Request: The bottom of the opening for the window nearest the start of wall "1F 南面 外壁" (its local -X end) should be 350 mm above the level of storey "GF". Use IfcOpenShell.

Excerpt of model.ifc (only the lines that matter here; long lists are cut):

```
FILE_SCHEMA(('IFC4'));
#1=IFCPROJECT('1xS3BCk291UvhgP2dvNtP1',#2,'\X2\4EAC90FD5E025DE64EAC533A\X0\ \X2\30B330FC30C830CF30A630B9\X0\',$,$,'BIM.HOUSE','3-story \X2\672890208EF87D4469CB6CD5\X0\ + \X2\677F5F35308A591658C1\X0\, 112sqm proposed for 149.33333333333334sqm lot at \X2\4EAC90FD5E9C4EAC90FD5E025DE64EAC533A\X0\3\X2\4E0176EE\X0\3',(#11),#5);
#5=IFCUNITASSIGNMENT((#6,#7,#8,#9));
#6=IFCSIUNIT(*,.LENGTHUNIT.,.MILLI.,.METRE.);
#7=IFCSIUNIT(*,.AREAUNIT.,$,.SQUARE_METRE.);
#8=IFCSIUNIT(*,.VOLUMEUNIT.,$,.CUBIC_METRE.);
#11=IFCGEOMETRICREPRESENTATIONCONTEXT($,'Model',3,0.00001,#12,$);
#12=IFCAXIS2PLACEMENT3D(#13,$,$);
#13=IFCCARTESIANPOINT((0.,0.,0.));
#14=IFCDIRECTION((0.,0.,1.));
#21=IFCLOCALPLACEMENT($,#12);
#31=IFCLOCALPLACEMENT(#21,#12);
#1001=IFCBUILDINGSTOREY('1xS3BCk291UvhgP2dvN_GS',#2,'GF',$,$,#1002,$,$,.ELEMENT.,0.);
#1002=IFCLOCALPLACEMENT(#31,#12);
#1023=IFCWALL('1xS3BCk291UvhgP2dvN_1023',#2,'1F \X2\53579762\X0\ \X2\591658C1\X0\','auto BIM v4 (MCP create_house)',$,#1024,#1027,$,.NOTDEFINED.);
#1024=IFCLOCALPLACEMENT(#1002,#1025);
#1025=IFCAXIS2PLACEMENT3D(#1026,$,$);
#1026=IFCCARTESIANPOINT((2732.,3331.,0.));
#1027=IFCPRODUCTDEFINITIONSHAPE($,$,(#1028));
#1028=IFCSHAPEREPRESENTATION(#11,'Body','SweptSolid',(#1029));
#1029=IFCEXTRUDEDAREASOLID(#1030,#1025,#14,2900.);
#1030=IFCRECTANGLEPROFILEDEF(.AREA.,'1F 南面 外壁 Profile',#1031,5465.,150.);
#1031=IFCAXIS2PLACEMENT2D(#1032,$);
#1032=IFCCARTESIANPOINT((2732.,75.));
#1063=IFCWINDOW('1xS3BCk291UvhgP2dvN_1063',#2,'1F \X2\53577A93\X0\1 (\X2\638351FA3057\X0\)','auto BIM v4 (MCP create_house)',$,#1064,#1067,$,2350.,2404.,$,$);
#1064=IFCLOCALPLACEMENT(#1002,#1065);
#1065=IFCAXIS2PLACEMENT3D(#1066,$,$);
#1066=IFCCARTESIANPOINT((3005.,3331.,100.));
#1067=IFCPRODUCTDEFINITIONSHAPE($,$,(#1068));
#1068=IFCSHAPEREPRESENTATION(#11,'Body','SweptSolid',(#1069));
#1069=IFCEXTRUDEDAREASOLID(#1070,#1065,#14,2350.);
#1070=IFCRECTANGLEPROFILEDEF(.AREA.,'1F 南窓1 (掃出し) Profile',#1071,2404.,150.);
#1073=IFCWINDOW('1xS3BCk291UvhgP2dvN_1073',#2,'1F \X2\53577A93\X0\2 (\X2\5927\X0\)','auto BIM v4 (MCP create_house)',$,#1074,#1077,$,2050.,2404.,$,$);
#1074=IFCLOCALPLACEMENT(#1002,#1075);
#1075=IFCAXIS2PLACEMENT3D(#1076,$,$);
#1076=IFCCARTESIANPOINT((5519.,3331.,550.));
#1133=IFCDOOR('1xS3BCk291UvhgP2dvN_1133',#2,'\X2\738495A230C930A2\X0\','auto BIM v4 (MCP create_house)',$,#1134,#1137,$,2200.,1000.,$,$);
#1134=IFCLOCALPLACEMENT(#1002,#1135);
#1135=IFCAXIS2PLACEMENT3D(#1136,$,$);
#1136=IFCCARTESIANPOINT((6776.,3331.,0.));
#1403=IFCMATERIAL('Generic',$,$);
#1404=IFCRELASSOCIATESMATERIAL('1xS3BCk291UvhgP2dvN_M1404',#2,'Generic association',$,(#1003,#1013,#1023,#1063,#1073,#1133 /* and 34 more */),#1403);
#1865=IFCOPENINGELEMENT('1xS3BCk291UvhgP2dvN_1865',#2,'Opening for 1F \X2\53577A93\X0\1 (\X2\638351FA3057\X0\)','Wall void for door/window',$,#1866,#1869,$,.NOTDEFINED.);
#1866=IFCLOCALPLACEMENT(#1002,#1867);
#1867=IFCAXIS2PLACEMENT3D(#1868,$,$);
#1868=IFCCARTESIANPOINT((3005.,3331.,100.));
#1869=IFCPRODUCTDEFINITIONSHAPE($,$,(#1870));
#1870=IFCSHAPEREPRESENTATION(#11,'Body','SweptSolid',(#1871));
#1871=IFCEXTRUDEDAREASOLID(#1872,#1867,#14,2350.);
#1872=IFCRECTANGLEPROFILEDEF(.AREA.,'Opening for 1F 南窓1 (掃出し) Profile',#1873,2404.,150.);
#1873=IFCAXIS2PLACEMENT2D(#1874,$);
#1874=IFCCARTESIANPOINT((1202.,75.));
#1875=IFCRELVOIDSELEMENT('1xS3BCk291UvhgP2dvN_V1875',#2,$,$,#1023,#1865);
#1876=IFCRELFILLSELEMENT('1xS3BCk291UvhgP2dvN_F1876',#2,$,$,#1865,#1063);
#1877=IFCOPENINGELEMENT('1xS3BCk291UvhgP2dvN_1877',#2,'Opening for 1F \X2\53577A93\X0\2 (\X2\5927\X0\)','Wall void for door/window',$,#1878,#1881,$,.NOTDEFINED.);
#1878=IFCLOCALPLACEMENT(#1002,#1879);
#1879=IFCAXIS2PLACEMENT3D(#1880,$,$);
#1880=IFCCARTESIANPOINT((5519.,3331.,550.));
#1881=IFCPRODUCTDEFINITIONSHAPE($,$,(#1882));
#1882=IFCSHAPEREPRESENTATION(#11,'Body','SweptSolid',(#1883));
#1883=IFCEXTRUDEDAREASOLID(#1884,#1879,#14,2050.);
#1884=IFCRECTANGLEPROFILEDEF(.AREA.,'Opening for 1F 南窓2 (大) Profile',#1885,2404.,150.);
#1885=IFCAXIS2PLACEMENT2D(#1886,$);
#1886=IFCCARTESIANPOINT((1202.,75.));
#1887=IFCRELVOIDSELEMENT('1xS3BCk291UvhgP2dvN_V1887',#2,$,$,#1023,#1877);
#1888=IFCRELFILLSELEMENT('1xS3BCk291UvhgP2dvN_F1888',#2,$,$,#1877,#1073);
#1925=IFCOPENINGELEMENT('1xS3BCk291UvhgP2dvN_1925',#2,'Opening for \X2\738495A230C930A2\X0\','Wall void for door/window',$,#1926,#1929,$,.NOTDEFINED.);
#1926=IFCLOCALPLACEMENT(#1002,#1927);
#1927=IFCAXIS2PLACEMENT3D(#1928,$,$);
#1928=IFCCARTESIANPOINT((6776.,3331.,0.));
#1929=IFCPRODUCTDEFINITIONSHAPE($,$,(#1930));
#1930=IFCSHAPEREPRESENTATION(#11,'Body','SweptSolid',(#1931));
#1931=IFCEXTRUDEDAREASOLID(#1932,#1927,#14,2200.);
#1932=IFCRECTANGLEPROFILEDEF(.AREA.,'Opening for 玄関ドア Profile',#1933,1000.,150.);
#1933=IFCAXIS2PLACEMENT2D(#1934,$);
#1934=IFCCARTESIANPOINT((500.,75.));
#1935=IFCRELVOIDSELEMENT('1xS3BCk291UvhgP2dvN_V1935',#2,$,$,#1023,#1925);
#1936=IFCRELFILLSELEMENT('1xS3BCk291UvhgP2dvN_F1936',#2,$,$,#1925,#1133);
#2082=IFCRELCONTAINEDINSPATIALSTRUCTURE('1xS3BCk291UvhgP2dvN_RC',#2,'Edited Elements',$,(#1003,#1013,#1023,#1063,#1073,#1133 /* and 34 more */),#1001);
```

```python
import numpy as np
import ifcopenshell
import ifcopenshell.api.geometry
import ifcopenshell.geom
import ifcopenshell.util.element
import ifcopenshell.util.placement
import ifcopenshell.util.shape
import ifcopenshell.util.unit

model = ifcopenshell.open("model.ifc")
unit_scale = ifcopenshell.util.unit.calculate_unit_scale(model)

window = model.by_guid("1xS3BCk291UvhgP2dvN_1063")
opening = window.FillsVoids[0].RelatingOpeningElement
storey = ifcopenshell.util.element.get_container(window, ifc_class="IfcBuildingStorey")
level = ifcopenshell.util.placement.get_local_placement(storey.ObjectPlacement)[2, 3]

# The opening's origin need not be at the sill, so measure its lowest point.
shape = ifcopenshell.geom.create_shape(ifcopenshell.geom.settings(), opening)
bottom = ifcopenshell.util.shape.get_shape_bottom_elevation(shape, shape.geometry) / unit_scale
dz = level + 0.35 / unit_scale - bottom

shift = np.array([0.0, 0.0, dz])
# The window is not placed relative to its opening, so move both.
for product in (opening, window):
    matrix = ifcopenshell.util.placement.get_local_placement(product.ObjectPlacement)
    matrix[:3, 3] += shift
    ifcopenshell.api.geometry.edit_object_placement(model, product=product, matrix=matrix, is_si=False)

print(f"moved by {dz * unit_scale:+.3f} m")

model.write("model-out.ifc")
```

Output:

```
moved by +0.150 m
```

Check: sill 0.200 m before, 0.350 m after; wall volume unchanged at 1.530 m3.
